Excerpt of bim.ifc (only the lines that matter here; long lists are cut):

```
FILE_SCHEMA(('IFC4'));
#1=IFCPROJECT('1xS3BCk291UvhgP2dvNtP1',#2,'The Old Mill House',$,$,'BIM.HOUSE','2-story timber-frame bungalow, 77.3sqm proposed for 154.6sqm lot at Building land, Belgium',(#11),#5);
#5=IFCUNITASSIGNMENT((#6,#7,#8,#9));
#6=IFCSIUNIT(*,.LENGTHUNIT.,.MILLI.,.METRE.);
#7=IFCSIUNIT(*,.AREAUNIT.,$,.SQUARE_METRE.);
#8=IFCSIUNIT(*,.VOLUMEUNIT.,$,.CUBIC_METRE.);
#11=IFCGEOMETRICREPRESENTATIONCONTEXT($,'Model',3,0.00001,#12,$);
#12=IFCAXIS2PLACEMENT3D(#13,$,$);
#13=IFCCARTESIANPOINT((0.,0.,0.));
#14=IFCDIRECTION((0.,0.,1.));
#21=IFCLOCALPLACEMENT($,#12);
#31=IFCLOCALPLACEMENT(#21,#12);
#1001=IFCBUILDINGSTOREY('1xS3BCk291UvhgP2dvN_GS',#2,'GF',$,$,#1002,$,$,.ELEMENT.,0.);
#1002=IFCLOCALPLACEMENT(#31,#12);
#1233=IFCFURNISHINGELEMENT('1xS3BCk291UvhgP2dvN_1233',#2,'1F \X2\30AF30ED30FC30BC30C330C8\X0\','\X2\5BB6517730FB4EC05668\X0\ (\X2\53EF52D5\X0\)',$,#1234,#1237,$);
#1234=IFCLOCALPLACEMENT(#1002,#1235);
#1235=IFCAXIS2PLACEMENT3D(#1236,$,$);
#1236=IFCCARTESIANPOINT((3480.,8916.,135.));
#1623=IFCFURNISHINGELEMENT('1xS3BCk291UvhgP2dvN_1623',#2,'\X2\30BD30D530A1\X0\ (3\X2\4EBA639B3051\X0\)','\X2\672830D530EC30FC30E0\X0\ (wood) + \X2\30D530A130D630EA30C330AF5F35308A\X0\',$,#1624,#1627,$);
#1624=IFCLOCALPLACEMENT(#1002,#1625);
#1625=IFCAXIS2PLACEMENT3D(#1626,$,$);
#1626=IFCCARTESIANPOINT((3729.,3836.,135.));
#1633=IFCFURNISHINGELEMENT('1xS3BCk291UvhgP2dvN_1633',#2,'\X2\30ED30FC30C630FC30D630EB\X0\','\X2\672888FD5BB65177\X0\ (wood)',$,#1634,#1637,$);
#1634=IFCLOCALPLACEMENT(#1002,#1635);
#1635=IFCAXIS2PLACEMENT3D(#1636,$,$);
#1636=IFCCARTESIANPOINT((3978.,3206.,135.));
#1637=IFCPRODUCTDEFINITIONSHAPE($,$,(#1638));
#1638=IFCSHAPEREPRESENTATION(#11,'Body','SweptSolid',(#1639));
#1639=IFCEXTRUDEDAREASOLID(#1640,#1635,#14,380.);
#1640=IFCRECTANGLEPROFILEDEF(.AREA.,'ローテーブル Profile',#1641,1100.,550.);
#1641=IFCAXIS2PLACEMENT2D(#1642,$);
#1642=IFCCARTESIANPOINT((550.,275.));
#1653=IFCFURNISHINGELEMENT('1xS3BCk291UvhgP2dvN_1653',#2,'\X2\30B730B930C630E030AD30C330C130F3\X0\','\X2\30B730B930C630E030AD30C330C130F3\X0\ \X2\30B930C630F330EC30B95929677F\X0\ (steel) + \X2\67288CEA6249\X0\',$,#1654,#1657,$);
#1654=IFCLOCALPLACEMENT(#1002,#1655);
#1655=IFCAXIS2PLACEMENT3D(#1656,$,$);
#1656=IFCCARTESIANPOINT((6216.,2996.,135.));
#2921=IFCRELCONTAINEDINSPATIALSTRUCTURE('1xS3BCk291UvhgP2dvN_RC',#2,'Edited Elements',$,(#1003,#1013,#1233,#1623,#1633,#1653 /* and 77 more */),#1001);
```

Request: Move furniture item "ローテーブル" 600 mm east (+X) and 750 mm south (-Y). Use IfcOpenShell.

```python
import ifcopenshell
import ifcopenshell.api.geometry
import ifcopenshell.util.placement

model = ifcopenshell.open("bim.ifc")

item = model.by_guid("1xS3BCk291UvhgP2dvN_1633")
matrix = ifcopenshell.util.placement.get_local_placement(item.ObjectPlacement)
matrix[0, 3] += 600.0
matrix[1, 3] -= 750.0
ifcopenshell.api.geometry.edit_object_placement(model, product=item, matrix=matrix, is_si=False)

print(ifcopenshell.util.placement.get_local_placement(item.ObjectPlacement).round(3) + 0.0)

model.write("bim_v2.ifc")
```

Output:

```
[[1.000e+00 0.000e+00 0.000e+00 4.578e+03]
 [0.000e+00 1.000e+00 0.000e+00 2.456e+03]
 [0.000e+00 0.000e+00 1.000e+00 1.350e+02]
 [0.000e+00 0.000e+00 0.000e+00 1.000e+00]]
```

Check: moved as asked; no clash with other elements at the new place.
